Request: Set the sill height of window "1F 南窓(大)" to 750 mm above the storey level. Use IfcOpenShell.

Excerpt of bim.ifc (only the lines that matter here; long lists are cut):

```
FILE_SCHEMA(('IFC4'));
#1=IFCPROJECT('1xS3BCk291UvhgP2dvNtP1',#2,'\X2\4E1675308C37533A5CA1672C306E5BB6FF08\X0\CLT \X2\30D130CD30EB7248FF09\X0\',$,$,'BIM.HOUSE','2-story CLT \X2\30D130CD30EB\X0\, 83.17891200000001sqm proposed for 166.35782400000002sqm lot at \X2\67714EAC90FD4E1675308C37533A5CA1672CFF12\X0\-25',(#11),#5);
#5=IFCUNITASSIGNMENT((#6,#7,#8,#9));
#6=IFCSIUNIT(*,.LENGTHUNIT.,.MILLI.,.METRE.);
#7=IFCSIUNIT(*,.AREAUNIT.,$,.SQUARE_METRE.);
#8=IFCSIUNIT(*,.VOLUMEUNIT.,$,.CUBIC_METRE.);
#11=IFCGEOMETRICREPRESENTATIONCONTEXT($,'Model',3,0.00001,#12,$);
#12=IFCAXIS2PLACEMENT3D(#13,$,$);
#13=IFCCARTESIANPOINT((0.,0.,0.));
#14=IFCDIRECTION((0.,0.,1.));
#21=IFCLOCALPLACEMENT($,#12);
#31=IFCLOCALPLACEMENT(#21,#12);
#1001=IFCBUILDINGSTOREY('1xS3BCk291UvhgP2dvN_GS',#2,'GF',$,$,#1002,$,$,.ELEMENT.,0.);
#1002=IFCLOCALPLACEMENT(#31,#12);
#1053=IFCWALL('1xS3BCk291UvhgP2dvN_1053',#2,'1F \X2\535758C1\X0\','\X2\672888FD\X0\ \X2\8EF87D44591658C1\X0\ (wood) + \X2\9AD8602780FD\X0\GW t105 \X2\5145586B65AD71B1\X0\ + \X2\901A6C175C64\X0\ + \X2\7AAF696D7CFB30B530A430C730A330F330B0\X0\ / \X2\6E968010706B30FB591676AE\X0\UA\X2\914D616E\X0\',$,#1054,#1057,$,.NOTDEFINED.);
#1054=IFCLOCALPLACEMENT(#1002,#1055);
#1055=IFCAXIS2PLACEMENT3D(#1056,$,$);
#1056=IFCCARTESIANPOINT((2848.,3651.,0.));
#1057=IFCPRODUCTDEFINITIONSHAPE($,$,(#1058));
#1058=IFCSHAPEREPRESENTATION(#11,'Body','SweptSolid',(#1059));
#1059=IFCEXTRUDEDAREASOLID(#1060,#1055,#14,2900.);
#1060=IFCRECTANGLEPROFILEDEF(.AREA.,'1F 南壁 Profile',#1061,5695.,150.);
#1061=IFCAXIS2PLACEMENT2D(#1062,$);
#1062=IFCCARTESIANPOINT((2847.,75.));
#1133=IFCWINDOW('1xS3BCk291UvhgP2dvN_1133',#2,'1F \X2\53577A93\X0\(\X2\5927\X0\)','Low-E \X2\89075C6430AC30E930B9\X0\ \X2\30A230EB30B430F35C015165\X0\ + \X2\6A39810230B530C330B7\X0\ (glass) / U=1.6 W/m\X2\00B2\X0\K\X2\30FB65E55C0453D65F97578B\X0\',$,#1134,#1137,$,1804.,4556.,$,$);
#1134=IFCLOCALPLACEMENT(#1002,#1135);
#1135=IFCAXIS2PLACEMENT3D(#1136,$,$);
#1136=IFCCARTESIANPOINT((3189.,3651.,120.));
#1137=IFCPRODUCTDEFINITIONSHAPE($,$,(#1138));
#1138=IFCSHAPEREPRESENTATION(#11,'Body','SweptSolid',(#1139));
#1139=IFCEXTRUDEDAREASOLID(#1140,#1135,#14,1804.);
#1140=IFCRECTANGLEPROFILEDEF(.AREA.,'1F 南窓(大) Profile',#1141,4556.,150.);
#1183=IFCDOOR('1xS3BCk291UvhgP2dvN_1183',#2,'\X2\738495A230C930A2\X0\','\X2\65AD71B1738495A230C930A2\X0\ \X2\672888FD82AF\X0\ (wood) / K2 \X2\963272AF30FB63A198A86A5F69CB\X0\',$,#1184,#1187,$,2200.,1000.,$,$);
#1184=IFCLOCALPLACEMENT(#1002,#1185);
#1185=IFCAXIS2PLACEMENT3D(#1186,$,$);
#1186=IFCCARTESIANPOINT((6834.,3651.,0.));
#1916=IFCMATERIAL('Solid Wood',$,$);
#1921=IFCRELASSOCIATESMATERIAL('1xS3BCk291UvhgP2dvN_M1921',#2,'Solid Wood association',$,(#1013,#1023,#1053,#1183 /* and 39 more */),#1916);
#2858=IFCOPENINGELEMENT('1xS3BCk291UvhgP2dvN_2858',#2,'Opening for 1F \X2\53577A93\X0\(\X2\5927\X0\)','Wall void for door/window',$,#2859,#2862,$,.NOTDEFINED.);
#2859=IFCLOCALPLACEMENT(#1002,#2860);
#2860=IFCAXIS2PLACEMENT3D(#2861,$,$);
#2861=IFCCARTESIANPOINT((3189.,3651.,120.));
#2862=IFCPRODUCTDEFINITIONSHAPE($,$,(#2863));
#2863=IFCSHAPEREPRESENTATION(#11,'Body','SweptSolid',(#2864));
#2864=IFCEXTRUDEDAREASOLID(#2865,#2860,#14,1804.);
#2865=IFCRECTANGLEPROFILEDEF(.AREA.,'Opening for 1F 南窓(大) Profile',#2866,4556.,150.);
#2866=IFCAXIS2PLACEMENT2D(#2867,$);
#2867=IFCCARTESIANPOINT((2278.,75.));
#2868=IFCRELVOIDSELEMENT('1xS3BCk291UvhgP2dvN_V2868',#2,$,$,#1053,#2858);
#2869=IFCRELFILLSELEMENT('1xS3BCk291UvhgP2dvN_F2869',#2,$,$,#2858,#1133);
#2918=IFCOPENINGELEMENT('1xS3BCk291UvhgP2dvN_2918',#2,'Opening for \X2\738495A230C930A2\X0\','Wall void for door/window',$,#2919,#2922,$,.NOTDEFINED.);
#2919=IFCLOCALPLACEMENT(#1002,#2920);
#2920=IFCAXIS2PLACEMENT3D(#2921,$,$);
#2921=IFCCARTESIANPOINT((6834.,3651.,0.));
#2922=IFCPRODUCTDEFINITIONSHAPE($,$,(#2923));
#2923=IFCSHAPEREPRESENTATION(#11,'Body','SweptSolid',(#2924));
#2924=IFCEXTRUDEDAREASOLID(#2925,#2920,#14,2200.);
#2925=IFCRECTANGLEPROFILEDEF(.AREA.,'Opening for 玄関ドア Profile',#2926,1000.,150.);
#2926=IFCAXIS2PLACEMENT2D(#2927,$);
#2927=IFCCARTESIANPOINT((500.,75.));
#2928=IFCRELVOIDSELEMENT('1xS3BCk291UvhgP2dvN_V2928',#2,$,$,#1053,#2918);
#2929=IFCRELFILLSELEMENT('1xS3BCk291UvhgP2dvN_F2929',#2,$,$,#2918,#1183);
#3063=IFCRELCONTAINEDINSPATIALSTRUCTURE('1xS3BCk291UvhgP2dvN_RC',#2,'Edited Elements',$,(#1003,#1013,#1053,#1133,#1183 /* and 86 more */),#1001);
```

```python
import numpy as np
import ifcopenshell
import ifcopenshell.api.geometry
import ifcopenshell.geom
import ifcopenshell.util.element
import ifcopenshell.util.placement
import ifcopenshell.util.shape
import ifcopenshell.util.unit

model = ifcopenshell.open("bim.ifc")
unit_scale = ifcopenshell.util.unit.calculate_unit_scale(model)

window = model.by_id(1133)
opening = window.FillsVoids[0].RelatingOpeningElement
storey = ifcopenshell.util.element.get_container(window, ifc_class="IfcBuildingStorey")
level = ifcopenshell.util.placement.get_local_placement(storey.ObjectPlacement)[2, 3]

# The opening's origin need not be at the sill, so measure its lowest point.
shape = ifcopenshell.geom.create_shape(ifcopenshell.geom.settings(), opening)
bottom = ifcopenshell.util.shape.get_shape_bottom_elevation(shape, shape.geometry) / unit_scale
dz = level + 0.75 / unit_scale - bottom

shift = np.array([0.0, 0.0, dz])
# The window is not placed relative to its opening, so move both.
for product in (opening, window):
    matrix = ifcopenshell.util.placement.get_local_placement(product.ObjectPlacement)
    matrix[:3, 3] += shift
    ifcopenshell.api.geometry.edit_object_placement(model, product=product, matrix=matrix, is_si=False)

print(f"moved by {dz * unit_scale:+.3f} m")

model.write("bim_edited.ifc")
```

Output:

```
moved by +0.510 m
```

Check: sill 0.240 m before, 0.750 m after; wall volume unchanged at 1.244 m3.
